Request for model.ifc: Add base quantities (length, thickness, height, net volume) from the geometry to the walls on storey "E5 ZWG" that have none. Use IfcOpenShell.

First a look at what the model holds.

```python
import ifcopenshell
import ifcopenshell.util.element
import ifcopenshell.util.unit

model = ifcopenshell.open("model.ifc")
print(model.schema)
for unit_type in ("LENGTHUNIT", "AREAUNIT", "VOLUMEUNIT"):
    print(unit_type, ifcopenshell.util.unit.calculate_unit_scale(model, unit_type))
storey = next(s for s in model.by_type("IfcBuildingStorey") if s.Name == "E5 ZWG")
walls = [e for e in ifcopenshell.util.element.get_decomposition(storey) if e.is_a("IfcWall")]
for e in sorted(walls, key=lambda e: e.id()):
    print(e.id(), e.is_a(), e.Name, list(ifcopenshell.util.element.get_psets(e, qtos_only=True)), sep=" | ")
```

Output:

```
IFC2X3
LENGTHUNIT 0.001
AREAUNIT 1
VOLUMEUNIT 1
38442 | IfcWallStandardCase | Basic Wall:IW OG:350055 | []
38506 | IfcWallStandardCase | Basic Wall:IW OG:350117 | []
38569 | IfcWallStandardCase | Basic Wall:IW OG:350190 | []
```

```python
import ifcopenshell
import ifcopenshell.api.pset
import ifcopenshell.geom
import ifcopenshell.util.element
import ifcopenshell.util.shape
import ifcopenshell.util.unit

model = ifcopenshell.open("model.ifc")
unit_scale = ifcopenshell.util.unit.calculate_unit_scale(model)
volume_scale = ifcopenshell.util.unit.calculate_unit_scale(model, "VOLUMEUNIT")
settings = ifcopenshell.geom.settings()

storey = next(s for s in model.by_type("IfcBuildingStorey") if s.Name == "E5 ZWG")
walls = [e for e in ifcopenshell.util.element.get_decomposition(storey) if e.is_a("IfcWall")]

for e in sorted(walls, key=lambda e: e.id()):
    if ifcopenshell.util.element.get_psets(e, qtos_only=True, should_inherit=False):
        continue
    # Geometry comes back in metres, in the element's own axes.
    shape = ifcopenshell.geom.create_shape(settings, e)
    values = {
        "Length": ifcopenshell.util.shape.get_x(shape.geometry) / unit_scale,
        "Width": ifcopenshell.util.shape.get_y(shape.geometry) / unit_scale,
        "Height": ifcopenshell.util.shape.get_z(shape.geometry) / unit_scale,
        "NetVolume": ifcopenshell.util.shape.get_volume(shape.geometry) / volume_scale,
    }
    qto = ifcopenshell.api.pset.add_qto(model, product=e, name="BaseQuantities")
    ifcopenshell.api.pset.edit_qto(model, qto=qto, properties=values)
    print(e.id(), {k: round(v, 3) for k, v in values.items()})

model.write("model_v2.ifc")
```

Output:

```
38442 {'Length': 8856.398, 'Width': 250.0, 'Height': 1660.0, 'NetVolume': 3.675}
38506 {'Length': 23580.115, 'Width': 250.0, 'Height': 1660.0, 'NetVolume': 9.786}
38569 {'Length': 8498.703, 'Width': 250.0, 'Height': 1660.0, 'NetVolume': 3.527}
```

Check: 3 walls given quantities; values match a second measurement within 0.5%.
